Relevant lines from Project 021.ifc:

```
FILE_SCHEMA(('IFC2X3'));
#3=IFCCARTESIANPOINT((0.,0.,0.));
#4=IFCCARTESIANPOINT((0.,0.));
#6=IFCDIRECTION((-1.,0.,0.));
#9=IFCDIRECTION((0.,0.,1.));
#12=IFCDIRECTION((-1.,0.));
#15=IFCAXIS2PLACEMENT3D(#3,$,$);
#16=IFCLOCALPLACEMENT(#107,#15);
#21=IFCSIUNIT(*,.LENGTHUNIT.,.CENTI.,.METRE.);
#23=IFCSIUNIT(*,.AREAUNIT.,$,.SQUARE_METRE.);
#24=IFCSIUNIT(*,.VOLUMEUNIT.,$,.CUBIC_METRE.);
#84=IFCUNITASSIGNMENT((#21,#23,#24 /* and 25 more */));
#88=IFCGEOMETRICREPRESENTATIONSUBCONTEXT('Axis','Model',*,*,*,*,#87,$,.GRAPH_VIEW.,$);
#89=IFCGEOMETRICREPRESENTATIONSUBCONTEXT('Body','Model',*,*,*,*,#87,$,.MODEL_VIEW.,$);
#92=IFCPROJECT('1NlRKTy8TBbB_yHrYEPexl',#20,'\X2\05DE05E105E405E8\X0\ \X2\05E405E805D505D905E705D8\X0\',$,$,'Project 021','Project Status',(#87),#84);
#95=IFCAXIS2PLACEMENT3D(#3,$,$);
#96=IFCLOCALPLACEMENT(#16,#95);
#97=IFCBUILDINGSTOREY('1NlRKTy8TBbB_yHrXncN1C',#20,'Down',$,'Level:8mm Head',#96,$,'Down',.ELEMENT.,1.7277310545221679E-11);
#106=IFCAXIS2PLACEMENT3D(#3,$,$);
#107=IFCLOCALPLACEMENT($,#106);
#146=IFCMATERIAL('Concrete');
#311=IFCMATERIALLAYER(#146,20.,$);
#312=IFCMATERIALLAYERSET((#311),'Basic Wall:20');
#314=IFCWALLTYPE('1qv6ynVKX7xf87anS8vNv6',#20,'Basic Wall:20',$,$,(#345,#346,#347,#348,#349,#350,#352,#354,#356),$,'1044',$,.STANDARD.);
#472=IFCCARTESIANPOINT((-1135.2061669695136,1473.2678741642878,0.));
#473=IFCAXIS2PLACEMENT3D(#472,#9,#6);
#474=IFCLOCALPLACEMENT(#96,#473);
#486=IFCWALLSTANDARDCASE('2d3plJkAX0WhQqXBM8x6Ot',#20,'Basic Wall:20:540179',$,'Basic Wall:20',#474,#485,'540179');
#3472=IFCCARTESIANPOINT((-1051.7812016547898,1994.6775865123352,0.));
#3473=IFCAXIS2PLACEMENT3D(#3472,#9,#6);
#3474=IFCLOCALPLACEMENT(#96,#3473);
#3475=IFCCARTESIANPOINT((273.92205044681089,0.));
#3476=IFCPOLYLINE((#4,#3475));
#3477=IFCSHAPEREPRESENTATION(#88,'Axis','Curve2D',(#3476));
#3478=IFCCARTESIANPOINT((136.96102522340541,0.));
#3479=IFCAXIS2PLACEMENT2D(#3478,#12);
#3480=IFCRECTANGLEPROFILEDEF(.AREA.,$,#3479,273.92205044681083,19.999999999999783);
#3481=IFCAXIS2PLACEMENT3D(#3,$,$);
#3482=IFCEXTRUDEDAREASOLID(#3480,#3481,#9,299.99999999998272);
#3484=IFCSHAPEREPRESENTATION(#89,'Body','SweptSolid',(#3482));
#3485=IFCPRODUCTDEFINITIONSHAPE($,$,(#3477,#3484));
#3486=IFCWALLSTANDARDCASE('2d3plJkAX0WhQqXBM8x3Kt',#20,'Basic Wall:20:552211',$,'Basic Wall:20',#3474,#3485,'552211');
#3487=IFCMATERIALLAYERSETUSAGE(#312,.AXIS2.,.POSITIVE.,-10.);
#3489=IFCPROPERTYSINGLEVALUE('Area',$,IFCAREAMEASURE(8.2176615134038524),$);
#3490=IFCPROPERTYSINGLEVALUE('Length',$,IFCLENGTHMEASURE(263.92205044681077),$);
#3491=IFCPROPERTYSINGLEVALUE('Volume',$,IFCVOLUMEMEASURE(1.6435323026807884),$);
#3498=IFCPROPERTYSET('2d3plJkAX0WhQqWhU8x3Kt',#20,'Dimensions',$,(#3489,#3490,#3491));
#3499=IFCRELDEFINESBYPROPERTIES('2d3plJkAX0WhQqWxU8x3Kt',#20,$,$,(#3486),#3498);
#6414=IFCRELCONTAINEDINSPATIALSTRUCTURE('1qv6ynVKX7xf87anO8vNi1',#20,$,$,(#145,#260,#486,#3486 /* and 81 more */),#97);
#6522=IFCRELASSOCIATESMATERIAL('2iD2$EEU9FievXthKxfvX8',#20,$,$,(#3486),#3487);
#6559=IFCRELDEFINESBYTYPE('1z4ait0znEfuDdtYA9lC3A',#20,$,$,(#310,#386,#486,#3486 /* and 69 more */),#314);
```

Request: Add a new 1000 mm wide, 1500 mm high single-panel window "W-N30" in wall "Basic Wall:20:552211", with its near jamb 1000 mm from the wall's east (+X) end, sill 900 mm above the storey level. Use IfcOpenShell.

```python
import numpy as np
import ifcopenshell
import ifcopenshell.api.feature
import ifcopenshell.api.geometry
import ifcopenshell.api.pset
import ifcopenshell.api.root
import ifcopenshell.api.spatial
import ifcopenshell.api.type
import ifcopenshell.geom
import ifcopenshell.util.element
import ifcopenshell.util.placement
import ifcopenshell.util.representation
import ifcopenshell.util.shape
import ifcopenshell.util.unit

model = ifcopenshell.open("Project 021.ifc")
unit_scale = ifcopenshell.util.unit.calculate_unit_scale(model)
area_scale = ifcopenshell.util.unit.calculate_unit_scale(model, "AREAUNIT")
volume_scale = ifcopenshell.util.unit.calculate_unit_scale(model, "VOLUMEUNIT")
settings = ifcopenshell.geom.settings()


def volume(element):
    """Net volume in cubic metres, openings subtracted."""
    shape = ifcopenshell.geom.create_shape(settings, element)
    return ifcopenshell.util.shape.get_volume(shape.geometry)


wall = model.by_guid("2d3plJkAX0WhQqXBM8x3Kt")
storey = ifcopenshell.util.element.get_container(wall, ifc_class="IfcBuildingStorey")
context = ifcopenshell.util.representation.get_context(model, "Model", "Body", "MODEL_VIEW")
before = volume(wall)

width, height, from_end, sill = 1, 1.5, 1, 0.9  # metres

# The wall runs along its own X axis, and the end named is its -X end.
wall_shape = ifcopenshell.geom.create_shape(settings, wall)
x, y, z = ifcopenshell.util.shape.get_vertices(wall_shape.geometry).T
start = x.min() + from_end
face, thickness = float(y.min()), float(y.max() - y.min())
wall_matrix = ifcopenshell.util.placement.get_local_placement(wall.ObjectPlacement)
level = ifcopenshell.util.placement.get_local_placement(storey.ObjectPlacement)[2, 3]


def in_wall(x, y):
    """Placement at x, y metres in the wall's axes, at sill height."""
    matrix = wall_matrix.copy()
    matrix[:, 3] = wall_matrix @ np.array([x / unit_scale, y / unit_scale, 0.0, 1.0])
    matrix[2, 3] = level + sill / unit_scale
    return matrix


# Opening: a box that overshoots both wall faces by 50 mm.
opening = ifcopenshell.api.root.create_entity(model, ifc_class="IfcOpeningElement")
box = ifcopenshell.api.geometry.add_wall_representation(
    model, context=context, length=width, height=height, thickness=thickness + 0.1
)
ifcopenshell.api.geometry.assign_representation(model, product=opening, representation=box)
ifcopenshell.api.geometry.edit_object_placement(model, product=opening, matrix=in_wall(start, face - 0.05), is_si=False)
ifcopenshell.api.feature.add_feature(model, feature=opening, element=wall)

window = ifcopenshell.api.root.create_entity(model, ifc_class="IfcWindow", name="W-N30")
window.OverallWidth, window.OverallHeight = width / unit_scale, height / unit_scale
body = ifcopenshell.api.geometry.add_window_representation(
    model,
    context=context,
    overall_width=window.OverallWidth,
    overall_height=window.OverallHeight,
    partition_type="SINGLE_PANEL",
)
ifcopenshell.api.geometry.assign_representation(model, product=window, representation=body)
ifcopenshell.api.spatial.assign_container(model, products=[window], relating_structure=storey)
fills = ifcopenshell.api.feature.add_filling(model, opening=opening, element=window)
fills.OwnerHistory = window.OwnerHistory  # required in IFC2X3

# IFC2X3 keeps the operation on the window style.
style = ifcopenshell.api.root.create_entity(model, ifc_class="IfcWindowStyle", name="W-N30")
style.OperationType, style.ConstructionType = "SINGLE_PANEL", "NOTDEFINED"
style.ParameterTakesPrecedence = style.Sizeable = False
ifcopenshell.api.type.assign_type(model, related_objects=[window], relating_type=style)

# Centre the window in the wall's thickness.
ifcopenshell.api.geometry.edit_object_placement(model, product=window, matrix=in_wall(start, face), is_si=False)
window_shape = ifcopenshell.geom.create_shape(settings, window)
depth = ifcopenshell.util.shape.get_vertices(window_shape.geometry)[:, 1]
offset = face + thickness / 2 - (depth.min() + depth.max()) / 2
ifcopenshell.api.geometry.edit_object_placement(model, product=window, matrix=in_wall(start, offset), is_si=False)

after = volume(wall)

# Update the wall's stored quantities.
pset = model.by_id(ifcopenshell.util.element.get_pset(wall, "Dimensions", should_inherit=False)["id"])
ifcopenshell.api.pset.edit_pset(model, pset=pset, properties={
    "Area": model.create_entity("IfcAreaMeasure", after / thickness / area_scale),
    "Volume": model.create_entity("IfcVolumeMeasure", after / volume_scale),
})

print(f"wall volume {before:.3f} -> {after:.3f} m3")

model.write("Project 021_rev.ifc")
```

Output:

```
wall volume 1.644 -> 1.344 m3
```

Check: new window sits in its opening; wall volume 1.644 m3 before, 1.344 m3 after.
